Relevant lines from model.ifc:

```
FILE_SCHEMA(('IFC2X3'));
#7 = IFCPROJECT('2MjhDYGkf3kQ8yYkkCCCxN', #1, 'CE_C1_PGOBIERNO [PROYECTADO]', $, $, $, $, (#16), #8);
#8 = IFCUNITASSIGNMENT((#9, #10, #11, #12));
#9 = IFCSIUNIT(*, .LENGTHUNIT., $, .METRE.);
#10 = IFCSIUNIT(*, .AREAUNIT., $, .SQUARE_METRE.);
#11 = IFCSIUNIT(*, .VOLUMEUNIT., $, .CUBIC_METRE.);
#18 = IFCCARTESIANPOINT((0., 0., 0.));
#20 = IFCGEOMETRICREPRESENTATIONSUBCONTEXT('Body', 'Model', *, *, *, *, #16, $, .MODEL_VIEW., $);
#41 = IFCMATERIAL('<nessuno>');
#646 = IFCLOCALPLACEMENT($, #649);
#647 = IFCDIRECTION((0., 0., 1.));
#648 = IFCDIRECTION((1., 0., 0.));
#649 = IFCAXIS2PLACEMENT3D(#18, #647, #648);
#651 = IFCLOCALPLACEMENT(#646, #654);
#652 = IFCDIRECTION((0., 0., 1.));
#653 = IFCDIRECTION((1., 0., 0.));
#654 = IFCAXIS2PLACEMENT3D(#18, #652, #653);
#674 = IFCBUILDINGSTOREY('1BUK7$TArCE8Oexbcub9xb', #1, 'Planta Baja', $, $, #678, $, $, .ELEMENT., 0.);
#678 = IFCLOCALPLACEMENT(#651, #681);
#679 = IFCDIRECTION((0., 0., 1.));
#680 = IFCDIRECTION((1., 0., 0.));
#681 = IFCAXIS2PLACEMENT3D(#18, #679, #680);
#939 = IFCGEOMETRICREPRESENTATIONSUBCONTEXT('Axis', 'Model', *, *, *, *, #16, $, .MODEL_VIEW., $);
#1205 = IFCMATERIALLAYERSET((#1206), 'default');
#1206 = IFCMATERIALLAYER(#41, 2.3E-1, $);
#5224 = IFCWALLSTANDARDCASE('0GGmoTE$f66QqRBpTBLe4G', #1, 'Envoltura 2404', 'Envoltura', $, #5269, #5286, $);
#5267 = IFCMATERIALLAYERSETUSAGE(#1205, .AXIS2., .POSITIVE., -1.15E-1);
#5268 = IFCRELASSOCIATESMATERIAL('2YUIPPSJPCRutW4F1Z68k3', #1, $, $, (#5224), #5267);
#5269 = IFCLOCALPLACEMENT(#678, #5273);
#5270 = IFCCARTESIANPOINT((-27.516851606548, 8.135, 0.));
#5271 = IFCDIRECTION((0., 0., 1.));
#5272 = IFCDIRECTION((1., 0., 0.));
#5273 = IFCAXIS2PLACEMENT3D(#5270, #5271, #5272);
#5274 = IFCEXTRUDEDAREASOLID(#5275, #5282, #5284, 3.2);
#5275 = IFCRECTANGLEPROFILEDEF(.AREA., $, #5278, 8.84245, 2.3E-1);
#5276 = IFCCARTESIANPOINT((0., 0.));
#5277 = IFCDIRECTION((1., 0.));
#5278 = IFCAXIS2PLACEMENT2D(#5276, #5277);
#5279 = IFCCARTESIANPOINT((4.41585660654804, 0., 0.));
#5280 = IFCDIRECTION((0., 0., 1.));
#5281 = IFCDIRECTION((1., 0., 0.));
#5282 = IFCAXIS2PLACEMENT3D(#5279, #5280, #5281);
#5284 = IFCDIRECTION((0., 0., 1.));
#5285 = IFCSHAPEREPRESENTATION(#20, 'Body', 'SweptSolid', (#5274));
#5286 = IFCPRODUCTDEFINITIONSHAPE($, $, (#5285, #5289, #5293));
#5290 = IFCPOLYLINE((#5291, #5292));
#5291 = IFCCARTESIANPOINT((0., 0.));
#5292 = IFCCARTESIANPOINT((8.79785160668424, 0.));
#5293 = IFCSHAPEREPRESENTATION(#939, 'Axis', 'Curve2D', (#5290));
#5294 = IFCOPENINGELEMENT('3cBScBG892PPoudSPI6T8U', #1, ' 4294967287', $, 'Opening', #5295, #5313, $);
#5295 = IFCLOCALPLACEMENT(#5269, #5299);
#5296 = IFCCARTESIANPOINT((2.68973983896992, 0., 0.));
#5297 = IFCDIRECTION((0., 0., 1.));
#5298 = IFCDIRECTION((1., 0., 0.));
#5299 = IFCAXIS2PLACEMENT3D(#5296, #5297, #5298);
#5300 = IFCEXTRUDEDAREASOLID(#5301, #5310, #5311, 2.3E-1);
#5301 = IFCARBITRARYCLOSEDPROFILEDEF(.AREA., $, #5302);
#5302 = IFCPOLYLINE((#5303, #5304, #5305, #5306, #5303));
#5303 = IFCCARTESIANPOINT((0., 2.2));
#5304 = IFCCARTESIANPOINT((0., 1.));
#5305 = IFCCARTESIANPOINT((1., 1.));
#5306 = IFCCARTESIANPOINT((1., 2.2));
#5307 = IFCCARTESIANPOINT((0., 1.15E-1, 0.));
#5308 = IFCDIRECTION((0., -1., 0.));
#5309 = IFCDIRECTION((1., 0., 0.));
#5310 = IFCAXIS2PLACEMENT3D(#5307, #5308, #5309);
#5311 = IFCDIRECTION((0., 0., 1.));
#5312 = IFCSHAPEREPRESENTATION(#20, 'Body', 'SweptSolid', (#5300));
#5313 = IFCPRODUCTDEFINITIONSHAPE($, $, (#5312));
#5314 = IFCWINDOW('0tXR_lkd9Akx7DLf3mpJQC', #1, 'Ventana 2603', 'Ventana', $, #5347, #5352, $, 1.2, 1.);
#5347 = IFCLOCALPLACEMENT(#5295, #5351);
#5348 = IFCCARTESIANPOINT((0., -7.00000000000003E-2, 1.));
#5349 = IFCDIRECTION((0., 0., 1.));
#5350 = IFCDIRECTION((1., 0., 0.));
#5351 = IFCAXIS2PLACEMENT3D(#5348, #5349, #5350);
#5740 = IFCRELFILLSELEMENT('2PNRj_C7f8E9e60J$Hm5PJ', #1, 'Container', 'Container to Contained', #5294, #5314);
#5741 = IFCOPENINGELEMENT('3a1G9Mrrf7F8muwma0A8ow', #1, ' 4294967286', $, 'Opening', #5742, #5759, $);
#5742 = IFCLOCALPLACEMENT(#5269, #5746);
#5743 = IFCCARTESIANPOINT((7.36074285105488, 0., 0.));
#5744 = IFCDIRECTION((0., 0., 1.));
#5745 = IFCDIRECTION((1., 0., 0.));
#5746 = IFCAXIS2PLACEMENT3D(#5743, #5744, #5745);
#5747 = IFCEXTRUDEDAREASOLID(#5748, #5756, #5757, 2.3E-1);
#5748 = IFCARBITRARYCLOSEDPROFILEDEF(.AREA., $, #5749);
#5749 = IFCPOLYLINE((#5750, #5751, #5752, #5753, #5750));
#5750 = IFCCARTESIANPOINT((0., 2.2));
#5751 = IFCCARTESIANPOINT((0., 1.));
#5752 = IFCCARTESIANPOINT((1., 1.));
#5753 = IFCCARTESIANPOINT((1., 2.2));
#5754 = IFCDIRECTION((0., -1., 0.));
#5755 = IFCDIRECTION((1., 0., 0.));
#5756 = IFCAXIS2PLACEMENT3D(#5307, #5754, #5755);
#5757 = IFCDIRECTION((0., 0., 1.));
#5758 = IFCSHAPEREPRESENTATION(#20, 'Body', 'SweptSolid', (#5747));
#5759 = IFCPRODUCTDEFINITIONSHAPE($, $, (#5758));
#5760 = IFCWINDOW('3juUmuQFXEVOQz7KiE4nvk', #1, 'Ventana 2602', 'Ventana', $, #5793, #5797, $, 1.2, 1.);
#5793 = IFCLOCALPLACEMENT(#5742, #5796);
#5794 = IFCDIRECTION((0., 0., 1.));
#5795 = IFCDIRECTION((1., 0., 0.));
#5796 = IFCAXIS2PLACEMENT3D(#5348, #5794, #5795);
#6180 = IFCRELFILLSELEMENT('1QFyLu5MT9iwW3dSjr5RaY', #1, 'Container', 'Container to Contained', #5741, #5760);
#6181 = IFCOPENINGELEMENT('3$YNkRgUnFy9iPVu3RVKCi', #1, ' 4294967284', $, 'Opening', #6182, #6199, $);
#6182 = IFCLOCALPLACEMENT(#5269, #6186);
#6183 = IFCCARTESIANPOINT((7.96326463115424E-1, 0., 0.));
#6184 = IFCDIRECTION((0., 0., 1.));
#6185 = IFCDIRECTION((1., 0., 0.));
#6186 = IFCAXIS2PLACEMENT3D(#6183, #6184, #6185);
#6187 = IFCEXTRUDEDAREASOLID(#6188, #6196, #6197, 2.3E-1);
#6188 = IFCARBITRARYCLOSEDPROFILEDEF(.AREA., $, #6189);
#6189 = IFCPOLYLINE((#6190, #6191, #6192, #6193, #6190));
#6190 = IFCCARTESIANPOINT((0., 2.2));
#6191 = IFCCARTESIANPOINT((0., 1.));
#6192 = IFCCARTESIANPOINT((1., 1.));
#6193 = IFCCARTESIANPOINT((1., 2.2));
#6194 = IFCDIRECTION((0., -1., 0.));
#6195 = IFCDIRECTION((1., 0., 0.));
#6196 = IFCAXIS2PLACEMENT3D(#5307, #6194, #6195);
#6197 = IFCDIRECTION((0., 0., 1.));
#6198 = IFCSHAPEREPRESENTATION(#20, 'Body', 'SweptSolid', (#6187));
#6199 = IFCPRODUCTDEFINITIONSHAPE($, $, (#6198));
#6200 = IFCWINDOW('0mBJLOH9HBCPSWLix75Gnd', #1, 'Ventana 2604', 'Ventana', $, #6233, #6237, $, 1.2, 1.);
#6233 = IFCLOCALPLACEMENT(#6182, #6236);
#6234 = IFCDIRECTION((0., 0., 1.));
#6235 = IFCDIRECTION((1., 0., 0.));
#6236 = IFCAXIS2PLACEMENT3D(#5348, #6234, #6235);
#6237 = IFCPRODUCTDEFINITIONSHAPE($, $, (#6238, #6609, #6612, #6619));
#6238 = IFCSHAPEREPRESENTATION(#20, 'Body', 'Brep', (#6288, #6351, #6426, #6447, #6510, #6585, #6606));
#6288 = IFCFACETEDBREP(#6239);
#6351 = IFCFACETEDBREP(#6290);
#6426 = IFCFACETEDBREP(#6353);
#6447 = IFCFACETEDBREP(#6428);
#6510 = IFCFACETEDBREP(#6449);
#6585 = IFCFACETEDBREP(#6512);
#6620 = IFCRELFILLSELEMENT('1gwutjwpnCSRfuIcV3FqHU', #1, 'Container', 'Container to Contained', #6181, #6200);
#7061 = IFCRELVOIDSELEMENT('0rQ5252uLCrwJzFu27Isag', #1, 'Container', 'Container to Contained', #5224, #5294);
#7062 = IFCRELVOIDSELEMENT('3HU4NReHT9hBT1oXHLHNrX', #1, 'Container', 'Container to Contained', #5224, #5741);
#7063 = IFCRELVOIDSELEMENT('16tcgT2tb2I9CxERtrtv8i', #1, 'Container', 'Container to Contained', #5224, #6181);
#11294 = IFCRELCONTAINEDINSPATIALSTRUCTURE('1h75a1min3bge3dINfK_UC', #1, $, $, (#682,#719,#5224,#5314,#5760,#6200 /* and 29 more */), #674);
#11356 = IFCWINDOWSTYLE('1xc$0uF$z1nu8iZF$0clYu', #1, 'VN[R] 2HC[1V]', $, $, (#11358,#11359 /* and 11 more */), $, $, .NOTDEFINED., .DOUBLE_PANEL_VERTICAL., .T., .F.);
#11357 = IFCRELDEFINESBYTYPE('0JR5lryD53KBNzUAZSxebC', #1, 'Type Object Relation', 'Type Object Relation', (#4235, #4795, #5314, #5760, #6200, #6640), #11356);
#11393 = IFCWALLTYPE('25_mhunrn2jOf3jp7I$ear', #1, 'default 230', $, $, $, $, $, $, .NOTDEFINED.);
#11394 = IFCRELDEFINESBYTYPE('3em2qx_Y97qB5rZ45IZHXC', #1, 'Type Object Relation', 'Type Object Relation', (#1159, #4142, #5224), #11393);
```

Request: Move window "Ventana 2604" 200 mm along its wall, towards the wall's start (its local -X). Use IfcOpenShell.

```python
import ifcopenshell
import ifcopenshell.api.geometry
import ifcopenshell.util.placement
import ifcopenshell.util.unit

model = ifcopenshell.open("model.ifc")
unit_scale = ifcopenshell.util.unit.calculate_unit_scale(model)

window = model.by_guid("0mBJLOH9HBCPSWLix75Gnd")
opening = window.FillsVoids[0].RelatingOpeningElement
wall = opening.VoidsElements[0].RelatingBuildingElement

wall_matrix = ifcopenshell.util.placement.get_local_placement(wall.ObjectPlacement)
shift = wall_matrix[:3, 0] * -0.2 / unit_scale
before = ifcopenshell.util.placement.get_local_placement(window.ObjectPlacement)[:3, 3].copy()

# The window is placed relative to its opening, so it follows when the opening moves.
matrix = ifcopenshell.util.placement.get_local_placement(opening.ObjectPlacement)
matrix[:3, 3] += shift
ifcopenshell.api.geometry.edit_object_placement(
    model, product=opening, matrix=matrix, is_si=False, should_transform_children=True
)

after = ifcopenshell.util.placement.get_local_placement(window.ObjectPlacement)[:3, 3]
print("window moved by", (after - before).round(3) + 0.0)

model.write("model_edited.ifc")
```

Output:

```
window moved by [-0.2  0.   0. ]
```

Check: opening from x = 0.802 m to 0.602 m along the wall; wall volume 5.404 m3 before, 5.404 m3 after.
